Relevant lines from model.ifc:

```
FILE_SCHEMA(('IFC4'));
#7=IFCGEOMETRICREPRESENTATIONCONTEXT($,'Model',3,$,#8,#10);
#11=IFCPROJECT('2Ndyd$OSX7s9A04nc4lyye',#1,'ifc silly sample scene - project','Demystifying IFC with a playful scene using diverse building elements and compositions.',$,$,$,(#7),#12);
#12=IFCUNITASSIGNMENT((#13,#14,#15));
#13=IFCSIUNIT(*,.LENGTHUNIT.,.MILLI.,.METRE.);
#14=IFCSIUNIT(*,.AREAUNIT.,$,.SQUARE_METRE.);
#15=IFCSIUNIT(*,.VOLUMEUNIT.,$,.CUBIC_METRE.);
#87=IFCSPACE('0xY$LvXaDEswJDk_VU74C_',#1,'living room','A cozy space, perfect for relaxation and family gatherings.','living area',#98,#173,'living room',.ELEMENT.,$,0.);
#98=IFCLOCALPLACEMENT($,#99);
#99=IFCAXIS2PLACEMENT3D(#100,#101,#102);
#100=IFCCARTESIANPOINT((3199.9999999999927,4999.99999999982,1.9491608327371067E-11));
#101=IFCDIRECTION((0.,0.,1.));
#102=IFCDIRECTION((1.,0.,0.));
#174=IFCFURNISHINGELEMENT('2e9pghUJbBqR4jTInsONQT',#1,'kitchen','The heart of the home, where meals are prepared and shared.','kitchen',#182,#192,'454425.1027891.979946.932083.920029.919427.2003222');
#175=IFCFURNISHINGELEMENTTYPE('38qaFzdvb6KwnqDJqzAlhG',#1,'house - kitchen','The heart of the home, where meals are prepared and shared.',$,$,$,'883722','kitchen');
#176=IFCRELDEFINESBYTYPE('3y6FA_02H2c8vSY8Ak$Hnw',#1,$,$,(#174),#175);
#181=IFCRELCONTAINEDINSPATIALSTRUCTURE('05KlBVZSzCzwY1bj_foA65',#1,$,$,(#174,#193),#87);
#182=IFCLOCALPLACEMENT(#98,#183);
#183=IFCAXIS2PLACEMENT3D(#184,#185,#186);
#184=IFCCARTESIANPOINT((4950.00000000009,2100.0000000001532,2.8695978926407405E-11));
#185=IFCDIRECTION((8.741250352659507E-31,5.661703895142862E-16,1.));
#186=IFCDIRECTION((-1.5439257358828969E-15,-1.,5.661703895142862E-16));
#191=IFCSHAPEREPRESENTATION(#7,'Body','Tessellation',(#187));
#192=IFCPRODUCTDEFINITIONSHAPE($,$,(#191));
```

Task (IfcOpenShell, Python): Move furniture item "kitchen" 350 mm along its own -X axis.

```python
import ifcopenshell
import ifcopenshell.api.geometry
import ifcopenshell.util.placement
import ifcopenshell.util.unit

model = ifcopenshell.open("model.ifc")
unit_scale = ifcopenshell.util.unit.calculate_unit_scale(model)

item = model.by_id(174)
matrix = ifcopenshell.util.placement.get_local_placement(item.ObjectPlacement)
matrix[:3, 3] -= matrix[:3, 0] * 0.35 / unit_scale
ifcopenshell.api.geometry.edit_object_placement(model, product=item, matrix=matrix, is_si=False)

print(ifcopenshell.util.placement.get_local_placement(item.ObjectPlacement).round(3) + 0.0)

model.write("model-out.ifc")
```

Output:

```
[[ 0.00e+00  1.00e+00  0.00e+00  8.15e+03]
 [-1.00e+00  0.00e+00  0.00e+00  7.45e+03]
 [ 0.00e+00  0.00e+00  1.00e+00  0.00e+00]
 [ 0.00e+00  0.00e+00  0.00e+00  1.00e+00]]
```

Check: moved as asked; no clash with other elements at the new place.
